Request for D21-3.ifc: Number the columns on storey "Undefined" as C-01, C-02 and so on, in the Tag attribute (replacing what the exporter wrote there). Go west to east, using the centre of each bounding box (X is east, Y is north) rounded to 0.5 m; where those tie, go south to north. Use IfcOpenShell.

First a look at what the model holds.

```python
import ifcopenshell
import ifcopenshell.util.element
import ifcopenshell.util.placement

model = ifcopenshell.open("D21-3.ifc")
print(model.schema)
storey = next(s for s in model.by_type("IfcBuildingStorey") if s.Name == "Undefined")
columns = [e for e in ifcopenshell.util.element.get_decomposition(storey) if e.is_a("IfcColumn")]
for e in sorted(columns, key=lambda e: e.id()):
    origin = ifcopenshell.util.placement.get_local_placement(e.ObjectPlacement)[:3, 3]
    print(e.id(), e.Tag, e.Name, origin.round(2) + 0.0, sep=" | ")
```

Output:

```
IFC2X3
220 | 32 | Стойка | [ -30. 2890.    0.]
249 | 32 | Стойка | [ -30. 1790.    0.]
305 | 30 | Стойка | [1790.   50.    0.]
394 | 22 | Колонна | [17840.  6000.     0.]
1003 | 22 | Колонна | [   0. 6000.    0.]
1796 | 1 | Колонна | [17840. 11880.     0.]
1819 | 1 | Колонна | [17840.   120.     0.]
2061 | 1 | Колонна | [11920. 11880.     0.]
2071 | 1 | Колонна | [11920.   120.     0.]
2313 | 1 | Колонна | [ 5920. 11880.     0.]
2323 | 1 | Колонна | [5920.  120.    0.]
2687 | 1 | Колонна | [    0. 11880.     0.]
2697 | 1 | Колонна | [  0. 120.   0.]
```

```python
import ifcopenshell
import ifcopenshell.geom
import ifcopenshell.util.element
import ifcopenshell.util.shape

model = ifcopenshell.open("D21-3.ifc")
settings = ifcopenshell.geom.settings()
settings.set("use-world-coords", True)


def centre(element):
    shape = ifcopenshell.geom.create_shape(settings, element)
    return ifcopenshell.util.shape.get_bbox_centroid(shape.geometry)


storey = next(s for s in model.by_type("IfcBuildingStorey") if s.Name == "Undefined")
columns = [e for e in ifcopenshell.util.element.get_decomposition(storey) if e.is_a("IfcColumn")]

# Insertion points can sit at a corner or the storey origin, so sort by the geometry (in metres).
centres = {e: centre(e) for e in columns}
columns.sort(key=lambda e: (round(centres[e][0] / 0.5), centres[e][1]))

for i, e in enumerate(columns, start=1):
    number = f"C-{i:02d}"
    e.Tag = number
    print(e.id(), number)

model.write("D21-3-out.ifc")
```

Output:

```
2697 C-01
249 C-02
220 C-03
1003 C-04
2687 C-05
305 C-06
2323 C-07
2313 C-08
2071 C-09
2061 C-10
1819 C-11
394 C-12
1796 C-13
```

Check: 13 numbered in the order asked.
